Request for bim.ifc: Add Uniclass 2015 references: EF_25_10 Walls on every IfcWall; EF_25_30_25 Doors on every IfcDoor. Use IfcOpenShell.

First a look at what the model holds.

```python
import ifcopenshell

model = ifcopenshell.open("bim.ifc")
print(model.schema)
print("classifications:", [c.Name for c in model.by_type("IfcClassification")])
for ifc_class in ("IfcDoor", "IfcRoof", "IfcStair", "IfcWall", "IfcWindow"):
    print(ifc_class, len(model.by_type(ifc_class)))
```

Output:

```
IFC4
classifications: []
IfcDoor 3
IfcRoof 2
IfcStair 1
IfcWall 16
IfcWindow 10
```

```python
import ifcopenshell
import ifcopenshell.api.classification

model = ifcopenshell.open("bim.ifc")

system = ifcopenshell.api.classification.add_classification(model, classification="Uniclass 2015")

codes = {
    "IfcWall": ("EF_25_10", "Walls"),
    "IfcDoor": ("EF_25_30_25", "Doors"),
}
for ifc_class, (code, name) in codes.items():
    products = model.by_type(ifc_class)
    ifcopenshell.api.classification.add_reference(
        model, products=products, classification=system, identification=code, name=name
    )
    print(code, len(products))

model.write("bim_edited.ifc")
```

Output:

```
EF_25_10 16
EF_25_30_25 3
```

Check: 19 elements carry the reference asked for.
